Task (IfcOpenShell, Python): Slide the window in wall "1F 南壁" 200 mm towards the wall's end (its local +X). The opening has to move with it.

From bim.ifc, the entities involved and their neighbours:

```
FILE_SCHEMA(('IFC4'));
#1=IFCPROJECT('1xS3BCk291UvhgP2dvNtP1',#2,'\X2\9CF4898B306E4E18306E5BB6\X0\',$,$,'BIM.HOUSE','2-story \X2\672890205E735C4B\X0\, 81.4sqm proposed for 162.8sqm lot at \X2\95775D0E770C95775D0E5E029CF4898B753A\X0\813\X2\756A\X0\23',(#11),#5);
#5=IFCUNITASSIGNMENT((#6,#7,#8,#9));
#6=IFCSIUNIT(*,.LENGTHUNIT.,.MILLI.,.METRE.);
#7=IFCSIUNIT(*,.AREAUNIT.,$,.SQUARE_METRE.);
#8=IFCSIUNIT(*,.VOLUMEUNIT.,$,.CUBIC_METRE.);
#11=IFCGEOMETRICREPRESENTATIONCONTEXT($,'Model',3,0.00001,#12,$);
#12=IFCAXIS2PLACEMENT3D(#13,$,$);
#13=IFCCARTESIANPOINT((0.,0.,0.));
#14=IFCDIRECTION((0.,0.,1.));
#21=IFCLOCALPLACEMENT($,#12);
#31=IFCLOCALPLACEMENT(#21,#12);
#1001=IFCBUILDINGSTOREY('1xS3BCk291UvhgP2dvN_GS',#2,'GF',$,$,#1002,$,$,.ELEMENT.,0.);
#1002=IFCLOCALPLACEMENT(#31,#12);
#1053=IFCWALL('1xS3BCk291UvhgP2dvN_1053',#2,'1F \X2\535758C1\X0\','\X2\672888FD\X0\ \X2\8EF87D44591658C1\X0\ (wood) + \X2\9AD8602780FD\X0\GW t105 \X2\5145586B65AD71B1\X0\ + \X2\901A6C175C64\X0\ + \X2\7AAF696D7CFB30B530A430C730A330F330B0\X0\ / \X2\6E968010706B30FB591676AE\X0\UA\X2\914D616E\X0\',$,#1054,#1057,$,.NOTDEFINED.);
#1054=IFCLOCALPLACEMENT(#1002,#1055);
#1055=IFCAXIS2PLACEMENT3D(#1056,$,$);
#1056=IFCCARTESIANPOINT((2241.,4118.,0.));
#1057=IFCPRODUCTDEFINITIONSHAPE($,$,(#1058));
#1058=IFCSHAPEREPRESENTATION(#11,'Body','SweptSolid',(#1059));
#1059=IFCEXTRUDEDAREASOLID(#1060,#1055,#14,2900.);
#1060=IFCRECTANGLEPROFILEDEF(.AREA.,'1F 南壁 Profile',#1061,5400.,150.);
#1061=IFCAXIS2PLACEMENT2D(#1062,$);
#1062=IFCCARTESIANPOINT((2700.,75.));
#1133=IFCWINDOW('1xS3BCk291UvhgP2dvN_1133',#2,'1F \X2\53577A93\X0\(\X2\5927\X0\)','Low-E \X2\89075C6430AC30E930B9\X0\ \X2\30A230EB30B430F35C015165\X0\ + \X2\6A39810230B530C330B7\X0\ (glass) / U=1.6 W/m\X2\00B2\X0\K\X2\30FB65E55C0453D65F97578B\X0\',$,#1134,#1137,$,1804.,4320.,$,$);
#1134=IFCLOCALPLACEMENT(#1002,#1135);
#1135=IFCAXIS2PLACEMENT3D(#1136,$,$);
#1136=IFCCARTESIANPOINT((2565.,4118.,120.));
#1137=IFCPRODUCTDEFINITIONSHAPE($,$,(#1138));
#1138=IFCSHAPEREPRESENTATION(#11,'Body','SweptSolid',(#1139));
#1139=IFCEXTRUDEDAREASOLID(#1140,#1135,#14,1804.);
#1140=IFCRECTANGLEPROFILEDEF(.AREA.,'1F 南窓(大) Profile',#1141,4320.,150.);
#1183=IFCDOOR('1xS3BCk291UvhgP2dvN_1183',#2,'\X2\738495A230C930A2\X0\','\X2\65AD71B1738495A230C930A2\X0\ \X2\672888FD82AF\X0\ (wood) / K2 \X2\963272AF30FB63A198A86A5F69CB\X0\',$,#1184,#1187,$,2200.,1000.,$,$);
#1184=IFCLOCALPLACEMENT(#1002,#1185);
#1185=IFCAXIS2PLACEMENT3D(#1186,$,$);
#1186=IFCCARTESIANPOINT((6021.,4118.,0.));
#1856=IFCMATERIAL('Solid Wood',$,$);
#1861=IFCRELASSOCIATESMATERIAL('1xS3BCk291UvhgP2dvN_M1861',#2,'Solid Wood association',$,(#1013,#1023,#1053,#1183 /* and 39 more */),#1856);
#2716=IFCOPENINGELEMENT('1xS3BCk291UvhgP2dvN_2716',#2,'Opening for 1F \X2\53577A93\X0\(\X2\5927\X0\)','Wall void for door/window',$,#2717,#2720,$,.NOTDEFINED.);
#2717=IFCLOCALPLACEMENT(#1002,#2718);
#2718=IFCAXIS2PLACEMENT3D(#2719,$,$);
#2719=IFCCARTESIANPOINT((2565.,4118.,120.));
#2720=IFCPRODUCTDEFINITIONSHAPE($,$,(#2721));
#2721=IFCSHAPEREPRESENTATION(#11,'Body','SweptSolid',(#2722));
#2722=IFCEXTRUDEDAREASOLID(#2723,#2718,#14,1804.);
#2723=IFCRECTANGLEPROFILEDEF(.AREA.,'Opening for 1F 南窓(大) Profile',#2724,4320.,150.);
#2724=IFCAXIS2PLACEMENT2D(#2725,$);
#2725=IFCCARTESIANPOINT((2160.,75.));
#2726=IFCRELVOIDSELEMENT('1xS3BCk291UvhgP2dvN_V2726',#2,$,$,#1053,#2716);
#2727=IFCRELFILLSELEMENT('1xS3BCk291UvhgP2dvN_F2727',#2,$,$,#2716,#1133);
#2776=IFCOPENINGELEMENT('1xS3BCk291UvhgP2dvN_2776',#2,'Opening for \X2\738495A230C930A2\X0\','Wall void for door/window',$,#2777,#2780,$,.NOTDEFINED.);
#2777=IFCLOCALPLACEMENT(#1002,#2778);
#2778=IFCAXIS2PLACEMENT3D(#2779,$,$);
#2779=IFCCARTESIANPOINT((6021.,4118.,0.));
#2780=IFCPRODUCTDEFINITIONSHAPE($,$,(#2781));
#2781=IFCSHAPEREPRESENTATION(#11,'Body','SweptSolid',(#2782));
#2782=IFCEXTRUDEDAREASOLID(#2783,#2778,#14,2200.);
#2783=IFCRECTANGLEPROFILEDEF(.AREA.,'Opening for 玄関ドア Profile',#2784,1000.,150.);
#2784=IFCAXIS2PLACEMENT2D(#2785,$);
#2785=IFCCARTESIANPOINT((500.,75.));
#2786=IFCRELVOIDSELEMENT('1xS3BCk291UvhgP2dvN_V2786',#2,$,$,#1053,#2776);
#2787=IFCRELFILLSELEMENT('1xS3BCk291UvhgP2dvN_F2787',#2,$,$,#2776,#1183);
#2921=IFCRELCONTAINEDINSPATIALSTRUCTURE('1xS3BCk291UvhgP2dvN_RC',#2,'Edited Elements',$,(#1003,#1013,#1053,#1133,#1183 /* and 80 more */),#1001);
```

```python
import ifcopenshell
import ifcopenshell.api.geometry
import ifcopenshell.util.placement
import ifcopenshell.util.unit

model = ifcopenshell.open("bim.ifc")
unit_scale = ifcopenshell.util.unit.calculate_unit_scale(model)

window = model.by_guid("1xS3BCk291UvhgP2dvN_1133")
opening = window.FillsVoids[0].RelatingOpeningElement
wall = opening.VoidsElements[0].RelatingBuildingElement

wall_matrix = ifcopenshell.util.placement.get_local_placement(wall.ObjectPlacement)
shift = wall_matrix[:3, 0] * 0.2 / unit_scale
before = ifcopenshell.util.placement.get_local_placement(window.ObjectPlacement)[:3, 3].copy()

# The window is not placed relative to its opening, so move both.
for product in (opening, window):
    matrix = ifcopenshell.util.placement.get_local_placement(product.ObjectPlacement)
    matrix[:3, 3] += shift
    ifcopenshell.api.geometry.edit_object_placement(model, product=product, matrix=matrix, is_si=False)

after = ifcopenshell.util.placement.get_local_placement(window.ObjectPlacement)[:3, 3]
print("window moved by", (after - before).round(3) + 0.0)

model.write("bim_updated.ifc")
```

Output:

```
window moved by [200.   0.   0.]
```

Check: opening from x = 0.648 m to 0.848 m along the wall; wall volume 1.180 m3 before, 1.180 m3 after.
